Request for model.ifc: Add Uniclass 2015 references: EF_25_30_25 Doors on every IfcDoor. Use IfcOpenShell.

First a look at what the model holds.

```python
import ifcopenshell

model = ifcopenshell.open("model.ifc")
print(model.schema)
print("classifications:", [c.Name for c in model.by_type("IfcClassification")])
for ifc_class in ("IfcDoor", "IfcRoof", "IfcStair", "IfcWall", "IfcWindow"):
    print(ifc_class, len(model.by_type(ifc_class)))
```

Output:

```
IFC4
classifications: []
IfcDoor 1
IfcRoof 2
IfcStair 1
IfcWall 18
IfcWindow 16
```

```python
import ifcopenshell
import ifcopenshell.api.classification

model = ifcopenshell.open("model.ifc")

system = ifcopenshell.api.classification.add_classification(model, classification="Uniclass 2015")

codes = {
    "IfcDoor": ("EF_25_30_25", "Doors"),
}
for ifc_class, (code, name) in codes.items():
    products = model.by_type(ifc_class)
    ifcopenshell.api.classification.add_reference(
        model, products=products, classification=system, identification=code, name=name
    )
    print(code, len(products))

model.write("model_rev.ifc")
```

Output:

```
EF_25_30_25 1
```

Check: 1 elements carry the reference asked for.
